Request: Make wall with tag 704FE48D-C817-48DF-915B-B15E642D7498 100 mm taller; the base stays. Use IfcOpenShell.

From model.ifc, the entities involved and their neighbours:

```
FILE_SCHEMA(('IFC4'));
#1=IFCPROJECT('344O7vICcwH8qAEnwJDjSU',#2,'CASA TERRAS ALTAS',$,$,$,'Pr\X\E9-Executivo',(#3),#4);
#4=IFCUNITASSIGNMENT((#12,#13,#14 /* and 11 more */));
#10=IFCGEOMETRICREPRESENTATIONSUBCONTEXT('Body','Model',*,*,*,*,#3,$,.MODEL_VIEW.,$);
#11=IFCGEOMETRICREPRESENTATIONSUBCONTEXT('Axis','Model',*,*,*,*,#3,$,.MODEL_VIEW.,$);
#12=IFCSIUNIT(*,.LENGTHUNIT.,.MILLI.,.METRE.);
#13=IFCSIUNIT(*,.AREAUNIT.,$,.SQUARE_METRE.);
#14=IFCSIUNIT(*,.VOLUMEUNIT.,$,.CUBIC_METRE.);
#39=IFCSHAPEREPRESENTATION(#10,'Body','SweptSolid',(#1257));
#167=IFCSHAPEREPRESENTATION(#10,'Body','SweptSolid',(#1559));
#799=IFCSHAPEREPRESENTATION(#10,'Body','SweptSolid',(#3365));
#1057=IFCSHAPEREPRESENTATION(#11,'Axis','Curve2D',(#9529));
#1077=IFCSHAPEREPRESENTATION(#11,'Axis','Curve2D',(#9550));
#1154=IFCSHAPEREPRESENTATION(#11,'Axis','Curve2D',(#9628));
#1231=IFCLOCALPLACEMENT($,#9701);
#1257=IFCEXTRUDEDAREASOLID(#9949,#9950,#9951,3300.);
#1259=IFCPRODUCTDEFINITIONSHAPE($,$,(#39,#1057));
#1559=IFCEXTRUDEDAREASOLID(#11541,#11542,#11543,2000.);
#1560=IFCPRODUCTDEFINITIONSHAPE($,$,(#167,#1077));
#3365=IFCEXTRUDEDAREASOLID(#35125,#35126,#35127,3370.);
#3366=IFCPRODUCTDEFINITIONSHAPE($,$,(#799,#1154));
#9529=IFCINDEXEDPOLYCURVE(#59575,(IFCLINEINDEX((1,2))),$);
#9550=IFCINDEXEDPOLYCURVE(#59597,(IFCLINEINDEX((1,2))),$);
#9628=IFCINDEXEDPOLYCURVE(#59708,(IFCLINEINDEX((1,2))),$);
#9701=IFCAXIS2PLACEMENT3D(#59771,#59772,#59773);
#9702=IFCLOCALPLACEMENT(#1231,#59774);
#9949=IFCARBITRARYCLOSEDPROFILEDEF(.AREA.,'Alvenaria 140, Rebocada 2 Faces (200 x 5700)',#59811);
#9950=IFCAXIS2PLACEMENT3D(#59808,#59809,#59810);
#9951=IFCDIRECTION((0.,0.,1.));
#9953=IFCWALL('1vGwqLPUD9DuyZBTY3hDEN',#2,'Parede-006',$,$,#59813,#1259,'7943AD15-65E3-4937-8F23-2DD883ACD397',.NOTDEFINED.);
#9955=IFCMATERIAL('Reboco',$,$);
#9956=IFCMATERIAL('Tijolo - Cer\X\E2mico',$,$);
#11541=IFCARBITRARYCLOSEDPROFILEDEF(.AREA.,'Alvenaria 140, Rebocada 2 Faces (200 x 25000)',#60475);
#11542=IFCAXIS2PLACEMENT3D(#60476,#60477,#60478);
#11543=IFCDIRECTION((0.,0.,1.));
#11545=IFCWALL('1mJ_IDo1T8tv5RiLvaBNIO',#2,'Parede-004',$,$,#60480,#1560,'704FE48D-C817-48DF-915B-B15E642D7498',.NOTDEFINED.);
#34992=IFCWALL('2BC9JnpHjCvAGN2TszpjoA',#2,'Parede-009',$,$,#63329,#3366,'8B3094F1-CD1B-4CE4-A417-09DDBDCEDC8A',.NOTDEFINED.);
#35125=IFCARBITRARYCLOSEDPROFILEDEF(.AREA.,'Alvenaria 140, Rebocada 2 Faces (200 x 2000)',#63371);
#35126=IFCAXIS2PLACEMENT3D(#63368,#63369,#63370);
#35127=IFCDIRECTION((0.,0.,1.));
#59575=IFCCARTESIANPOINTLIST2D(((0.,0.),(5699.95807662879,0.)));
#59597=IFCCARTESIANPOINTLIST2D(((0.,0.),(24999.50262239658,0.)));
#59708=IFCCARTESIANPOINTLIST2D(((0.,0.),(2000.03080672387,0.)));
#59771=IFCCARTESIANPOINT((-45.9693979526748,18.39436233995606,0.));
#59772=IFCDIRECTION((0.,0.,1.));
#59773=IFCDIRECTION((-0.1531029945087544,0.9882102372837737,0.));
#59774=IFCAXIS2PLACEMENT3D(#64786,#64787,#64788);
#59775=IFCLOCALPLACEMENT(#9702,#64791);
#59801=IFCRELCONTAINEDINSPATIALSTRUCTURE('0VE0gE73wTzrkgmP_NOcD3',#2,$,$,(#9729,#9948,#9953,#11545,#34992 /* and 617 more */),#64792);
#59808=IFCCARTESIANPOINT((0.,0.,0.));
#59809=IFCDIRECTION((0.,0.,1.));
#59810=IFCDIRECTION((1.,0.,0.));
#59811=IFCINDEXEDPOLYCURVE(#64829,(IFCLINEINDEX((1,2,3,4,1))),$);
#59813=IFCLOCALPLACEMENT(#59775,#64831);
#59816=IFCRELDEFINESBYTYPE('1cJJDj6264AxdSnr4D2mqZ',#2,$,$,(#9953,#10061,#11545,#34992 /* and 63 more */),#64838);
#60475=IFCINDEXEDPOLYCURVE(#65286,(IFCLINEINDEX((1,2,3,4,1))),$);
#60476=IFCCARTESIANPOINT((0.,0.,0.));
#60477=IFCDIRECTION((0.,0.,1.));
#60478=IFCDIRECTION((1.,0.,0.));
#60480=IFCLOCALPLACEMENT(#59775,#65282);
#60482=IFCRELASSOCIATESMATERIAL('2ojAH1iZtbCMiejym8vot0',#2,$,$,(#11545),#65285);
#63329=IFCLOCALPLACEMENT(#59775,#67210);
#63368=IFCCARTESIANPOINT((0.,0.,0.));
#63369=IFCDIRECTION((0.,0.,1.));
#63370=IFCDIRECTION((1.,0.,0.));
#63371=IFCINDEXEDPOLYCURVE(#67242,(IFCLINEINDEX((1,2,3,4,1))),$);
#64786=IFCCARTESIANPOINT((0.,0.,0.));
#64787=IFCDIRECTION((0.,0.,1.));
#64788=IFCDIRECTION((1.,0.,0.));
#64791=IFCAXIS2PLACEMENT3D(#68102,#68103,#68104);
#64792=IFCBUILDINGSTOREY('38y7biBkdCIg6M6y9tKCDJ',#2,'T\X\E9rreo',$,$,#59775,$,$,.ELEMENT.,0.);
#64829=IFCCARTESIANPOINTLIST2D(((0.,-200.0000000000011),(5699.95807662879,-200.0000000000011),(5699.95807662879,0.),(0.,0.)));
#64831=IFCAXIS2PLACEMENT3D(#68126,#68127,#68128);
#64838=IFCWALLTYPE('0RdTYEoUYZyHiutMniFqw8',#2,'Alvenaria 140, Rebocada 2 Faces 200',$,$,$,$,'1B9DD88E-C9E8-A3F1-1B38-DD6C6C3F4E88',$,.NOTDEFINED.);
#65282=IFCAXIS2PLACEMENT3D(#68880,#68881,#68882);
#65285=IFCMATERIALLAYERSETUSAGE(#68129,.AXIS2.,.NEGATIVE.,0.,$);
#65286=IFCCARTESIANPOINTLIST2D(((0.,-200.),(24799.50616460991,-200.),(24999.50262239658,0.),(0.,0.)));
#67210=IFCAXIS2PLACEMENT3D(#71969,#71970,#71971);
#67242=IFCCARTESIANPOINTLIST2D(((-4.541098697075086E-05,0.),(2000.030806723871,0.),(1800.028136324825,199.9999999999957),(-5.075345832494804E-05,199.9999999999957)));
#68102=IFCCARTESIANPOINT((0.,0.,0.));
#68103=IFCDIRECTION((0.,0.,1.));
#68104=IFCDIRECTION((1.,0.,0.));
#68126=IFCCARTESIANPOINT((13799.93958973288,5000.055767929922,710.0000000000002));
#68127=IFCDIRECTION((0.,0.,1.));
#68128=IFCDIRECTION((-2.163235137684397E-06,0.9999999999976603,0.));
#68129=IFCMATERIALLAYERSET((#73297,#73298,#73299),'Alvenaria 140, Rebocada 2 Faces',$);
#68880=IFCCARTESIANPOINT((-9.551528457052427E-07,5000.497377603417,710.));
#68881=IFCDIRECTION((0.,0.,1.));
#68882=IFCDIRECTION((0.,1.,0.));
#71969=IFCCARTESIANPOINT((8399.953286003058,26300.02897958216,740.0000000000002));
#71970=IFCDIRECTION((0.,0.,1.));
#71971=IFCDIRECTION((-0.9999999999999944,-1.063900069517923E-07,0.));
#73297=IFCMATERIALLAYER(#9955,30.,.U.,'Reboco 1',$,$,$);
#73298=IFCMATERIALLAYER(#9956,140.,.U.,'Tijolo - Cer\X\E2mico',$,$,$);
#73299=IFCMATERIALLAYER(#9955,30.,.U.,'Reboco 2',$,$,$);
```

```python
import ifcopenshell
import ifcopenshell.geom
import ifcopenshell.util.representation
import ifcopenshell.util.shape

model = ifcopenshell.open("model.ifc")
settings = ifcopenshell.geom.settings()


def volume(element):
    """Net volume in cubic metres, openings subtracted."""
    shape = ifcopenshell.geom.create_shape(settings, element)
    return ifcopenshell.util.shape.get_volume(shape.geometry)


wall = model.by_id(11545)
before = volume(wall)

body = ifcopenshell.util.representation.get_representation(wall, "Model", "Body")
solid = body.Items[0]
old_height = solid.Depth
solid.Depth += 100.0
after = volume(wall)

print(f"height {old_height:g} -> {solid.Depth:g}, volume {before:.3f} -> {after:.3f} m3")

model.write("model_edited.ifc")
```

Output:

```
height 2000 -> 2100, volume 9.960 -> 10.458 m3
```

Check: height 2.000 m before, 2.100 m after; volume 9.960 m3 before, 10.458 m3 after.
